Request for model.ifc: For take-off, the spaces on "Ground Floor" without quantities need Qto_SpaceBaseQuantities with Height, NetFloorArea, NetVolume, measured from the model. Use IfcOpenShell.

First a look at what the model holds.

```python
import ifcopenshell
import ifcopenshell.util.element
import ifcopenshell.util.unit

model = ifcopenshell.open("model.ifc")
print(model.schema)
for unit_type in ("LENGTHUNIT", "AREAUNIT", "VOLUMEUNIT"):
    print(unit_type, ifcopenshell.util.unit.calculate_unit_scale(model, unit_type))
storey = next(s for s in model.by_type("IfcBuildingStorey") if s.Name == "Ground Floor")
spaces = [e for e in ifcopenshell.util.element.get_decomposition(storey) if e.is_a("IfcSpace")]
for e in sorted(spaces, key=lambda e: e.id()):
    print(e.id(), e.is_a(), e.Name, list(ifcopenshell.util.element.get_psets(e, qtos_only=True)), sep=" | ")
```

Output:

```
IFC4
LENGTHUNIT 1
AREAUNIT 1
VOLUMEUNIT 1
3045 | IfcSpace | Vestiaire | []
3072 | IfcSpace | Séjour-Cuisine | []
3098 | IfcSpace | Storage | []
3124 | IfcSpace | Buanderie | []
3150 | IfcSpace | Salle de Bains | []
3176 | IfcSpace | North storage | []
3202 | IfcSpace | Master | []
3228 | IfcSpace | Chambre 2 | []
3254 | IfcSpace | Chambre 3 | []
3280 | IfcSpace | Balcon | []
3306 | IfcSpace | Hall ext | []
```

```python
import ifcopenshell
import ifcopenshell.api.pset
import ifcopenshell.geom
import ifcopenshell.util.element
import ifcopenshell.util.shape
import ifcopenshell.util.unit

model = ifcopenshell.open("model.ifc")
unit_scale = ifcopenshell.util.unit.calculate_unit_scale(model)
area_scale = ifcopenshell.util.unit.calculate_unit_scale(model, "AREAUNIT")
volume_scale = ifcopenshell.util.unit.calculate_unit_scale(model, "VOLUMEUNIT")
settings = ifcopenshell.geom.settings()

storey = next(s for s in model.by_type("IfcBuildingStorey") if s.Name == "Ground Floor")
spaces = [e for e in ifcopenshell.util.element.get_decomposition(storey) if e.is_a("IfcSpace")]

for e in sorted(spaces, key=lambda e: e.id()):
    if ifcopenshell.util.element.get_psets(e, qtos_only=True, should_inherit=False):
        continue
    # Geometry comes back in metres, in the element's own axes.
    shape = ifcopenshell.geom.create_shape(settings, e)
    values = {
        "Height": ifcopenshell.util.shape.get_z(shape.geometry) / unit_scale,
        "NetFloorArea": ifcopenshell.util.shape.get_footprint_area(shape.geometry) / area_scale,
        "NetVolume": ifcopenshell.util.shape.get_volume(shape.geometry) / volume_scale,
    }
    qto = ifcopenshell.api.pset.add_qto(model, product=e, name="Qto_SpaceBaseQuantities")
    ifcopenshell.api.pset.edit_qto(model, qto=qto, properties=values)
    print(e.id(), {k: round(v, 3) for k, v in values.items()})

model.write("model_updated.ifc")
```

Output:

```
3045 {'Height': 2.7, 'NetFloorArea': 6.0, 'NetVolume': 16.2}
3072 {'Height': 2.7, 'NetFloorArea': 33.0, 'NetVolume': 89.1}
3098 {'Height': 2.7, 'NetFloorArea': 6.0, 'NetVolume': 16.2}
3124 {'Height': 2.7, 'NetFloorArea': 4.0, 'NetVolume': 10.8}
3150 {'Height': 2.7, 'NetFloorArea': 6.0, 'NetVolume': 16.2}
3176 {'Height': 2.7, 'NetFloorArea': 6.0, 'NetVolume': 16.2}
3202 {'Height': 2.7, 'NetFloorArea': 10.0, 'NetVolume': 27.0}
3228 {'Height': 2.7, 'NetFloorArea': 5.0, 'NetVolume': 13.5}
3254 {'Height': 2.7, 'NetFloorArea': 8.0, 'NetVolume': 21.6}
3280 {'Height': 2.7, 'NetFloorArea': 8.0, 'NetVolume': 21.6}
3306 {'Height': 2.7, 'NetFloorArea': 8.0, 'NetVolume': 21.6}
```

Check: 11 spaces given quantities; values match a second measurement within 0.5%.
